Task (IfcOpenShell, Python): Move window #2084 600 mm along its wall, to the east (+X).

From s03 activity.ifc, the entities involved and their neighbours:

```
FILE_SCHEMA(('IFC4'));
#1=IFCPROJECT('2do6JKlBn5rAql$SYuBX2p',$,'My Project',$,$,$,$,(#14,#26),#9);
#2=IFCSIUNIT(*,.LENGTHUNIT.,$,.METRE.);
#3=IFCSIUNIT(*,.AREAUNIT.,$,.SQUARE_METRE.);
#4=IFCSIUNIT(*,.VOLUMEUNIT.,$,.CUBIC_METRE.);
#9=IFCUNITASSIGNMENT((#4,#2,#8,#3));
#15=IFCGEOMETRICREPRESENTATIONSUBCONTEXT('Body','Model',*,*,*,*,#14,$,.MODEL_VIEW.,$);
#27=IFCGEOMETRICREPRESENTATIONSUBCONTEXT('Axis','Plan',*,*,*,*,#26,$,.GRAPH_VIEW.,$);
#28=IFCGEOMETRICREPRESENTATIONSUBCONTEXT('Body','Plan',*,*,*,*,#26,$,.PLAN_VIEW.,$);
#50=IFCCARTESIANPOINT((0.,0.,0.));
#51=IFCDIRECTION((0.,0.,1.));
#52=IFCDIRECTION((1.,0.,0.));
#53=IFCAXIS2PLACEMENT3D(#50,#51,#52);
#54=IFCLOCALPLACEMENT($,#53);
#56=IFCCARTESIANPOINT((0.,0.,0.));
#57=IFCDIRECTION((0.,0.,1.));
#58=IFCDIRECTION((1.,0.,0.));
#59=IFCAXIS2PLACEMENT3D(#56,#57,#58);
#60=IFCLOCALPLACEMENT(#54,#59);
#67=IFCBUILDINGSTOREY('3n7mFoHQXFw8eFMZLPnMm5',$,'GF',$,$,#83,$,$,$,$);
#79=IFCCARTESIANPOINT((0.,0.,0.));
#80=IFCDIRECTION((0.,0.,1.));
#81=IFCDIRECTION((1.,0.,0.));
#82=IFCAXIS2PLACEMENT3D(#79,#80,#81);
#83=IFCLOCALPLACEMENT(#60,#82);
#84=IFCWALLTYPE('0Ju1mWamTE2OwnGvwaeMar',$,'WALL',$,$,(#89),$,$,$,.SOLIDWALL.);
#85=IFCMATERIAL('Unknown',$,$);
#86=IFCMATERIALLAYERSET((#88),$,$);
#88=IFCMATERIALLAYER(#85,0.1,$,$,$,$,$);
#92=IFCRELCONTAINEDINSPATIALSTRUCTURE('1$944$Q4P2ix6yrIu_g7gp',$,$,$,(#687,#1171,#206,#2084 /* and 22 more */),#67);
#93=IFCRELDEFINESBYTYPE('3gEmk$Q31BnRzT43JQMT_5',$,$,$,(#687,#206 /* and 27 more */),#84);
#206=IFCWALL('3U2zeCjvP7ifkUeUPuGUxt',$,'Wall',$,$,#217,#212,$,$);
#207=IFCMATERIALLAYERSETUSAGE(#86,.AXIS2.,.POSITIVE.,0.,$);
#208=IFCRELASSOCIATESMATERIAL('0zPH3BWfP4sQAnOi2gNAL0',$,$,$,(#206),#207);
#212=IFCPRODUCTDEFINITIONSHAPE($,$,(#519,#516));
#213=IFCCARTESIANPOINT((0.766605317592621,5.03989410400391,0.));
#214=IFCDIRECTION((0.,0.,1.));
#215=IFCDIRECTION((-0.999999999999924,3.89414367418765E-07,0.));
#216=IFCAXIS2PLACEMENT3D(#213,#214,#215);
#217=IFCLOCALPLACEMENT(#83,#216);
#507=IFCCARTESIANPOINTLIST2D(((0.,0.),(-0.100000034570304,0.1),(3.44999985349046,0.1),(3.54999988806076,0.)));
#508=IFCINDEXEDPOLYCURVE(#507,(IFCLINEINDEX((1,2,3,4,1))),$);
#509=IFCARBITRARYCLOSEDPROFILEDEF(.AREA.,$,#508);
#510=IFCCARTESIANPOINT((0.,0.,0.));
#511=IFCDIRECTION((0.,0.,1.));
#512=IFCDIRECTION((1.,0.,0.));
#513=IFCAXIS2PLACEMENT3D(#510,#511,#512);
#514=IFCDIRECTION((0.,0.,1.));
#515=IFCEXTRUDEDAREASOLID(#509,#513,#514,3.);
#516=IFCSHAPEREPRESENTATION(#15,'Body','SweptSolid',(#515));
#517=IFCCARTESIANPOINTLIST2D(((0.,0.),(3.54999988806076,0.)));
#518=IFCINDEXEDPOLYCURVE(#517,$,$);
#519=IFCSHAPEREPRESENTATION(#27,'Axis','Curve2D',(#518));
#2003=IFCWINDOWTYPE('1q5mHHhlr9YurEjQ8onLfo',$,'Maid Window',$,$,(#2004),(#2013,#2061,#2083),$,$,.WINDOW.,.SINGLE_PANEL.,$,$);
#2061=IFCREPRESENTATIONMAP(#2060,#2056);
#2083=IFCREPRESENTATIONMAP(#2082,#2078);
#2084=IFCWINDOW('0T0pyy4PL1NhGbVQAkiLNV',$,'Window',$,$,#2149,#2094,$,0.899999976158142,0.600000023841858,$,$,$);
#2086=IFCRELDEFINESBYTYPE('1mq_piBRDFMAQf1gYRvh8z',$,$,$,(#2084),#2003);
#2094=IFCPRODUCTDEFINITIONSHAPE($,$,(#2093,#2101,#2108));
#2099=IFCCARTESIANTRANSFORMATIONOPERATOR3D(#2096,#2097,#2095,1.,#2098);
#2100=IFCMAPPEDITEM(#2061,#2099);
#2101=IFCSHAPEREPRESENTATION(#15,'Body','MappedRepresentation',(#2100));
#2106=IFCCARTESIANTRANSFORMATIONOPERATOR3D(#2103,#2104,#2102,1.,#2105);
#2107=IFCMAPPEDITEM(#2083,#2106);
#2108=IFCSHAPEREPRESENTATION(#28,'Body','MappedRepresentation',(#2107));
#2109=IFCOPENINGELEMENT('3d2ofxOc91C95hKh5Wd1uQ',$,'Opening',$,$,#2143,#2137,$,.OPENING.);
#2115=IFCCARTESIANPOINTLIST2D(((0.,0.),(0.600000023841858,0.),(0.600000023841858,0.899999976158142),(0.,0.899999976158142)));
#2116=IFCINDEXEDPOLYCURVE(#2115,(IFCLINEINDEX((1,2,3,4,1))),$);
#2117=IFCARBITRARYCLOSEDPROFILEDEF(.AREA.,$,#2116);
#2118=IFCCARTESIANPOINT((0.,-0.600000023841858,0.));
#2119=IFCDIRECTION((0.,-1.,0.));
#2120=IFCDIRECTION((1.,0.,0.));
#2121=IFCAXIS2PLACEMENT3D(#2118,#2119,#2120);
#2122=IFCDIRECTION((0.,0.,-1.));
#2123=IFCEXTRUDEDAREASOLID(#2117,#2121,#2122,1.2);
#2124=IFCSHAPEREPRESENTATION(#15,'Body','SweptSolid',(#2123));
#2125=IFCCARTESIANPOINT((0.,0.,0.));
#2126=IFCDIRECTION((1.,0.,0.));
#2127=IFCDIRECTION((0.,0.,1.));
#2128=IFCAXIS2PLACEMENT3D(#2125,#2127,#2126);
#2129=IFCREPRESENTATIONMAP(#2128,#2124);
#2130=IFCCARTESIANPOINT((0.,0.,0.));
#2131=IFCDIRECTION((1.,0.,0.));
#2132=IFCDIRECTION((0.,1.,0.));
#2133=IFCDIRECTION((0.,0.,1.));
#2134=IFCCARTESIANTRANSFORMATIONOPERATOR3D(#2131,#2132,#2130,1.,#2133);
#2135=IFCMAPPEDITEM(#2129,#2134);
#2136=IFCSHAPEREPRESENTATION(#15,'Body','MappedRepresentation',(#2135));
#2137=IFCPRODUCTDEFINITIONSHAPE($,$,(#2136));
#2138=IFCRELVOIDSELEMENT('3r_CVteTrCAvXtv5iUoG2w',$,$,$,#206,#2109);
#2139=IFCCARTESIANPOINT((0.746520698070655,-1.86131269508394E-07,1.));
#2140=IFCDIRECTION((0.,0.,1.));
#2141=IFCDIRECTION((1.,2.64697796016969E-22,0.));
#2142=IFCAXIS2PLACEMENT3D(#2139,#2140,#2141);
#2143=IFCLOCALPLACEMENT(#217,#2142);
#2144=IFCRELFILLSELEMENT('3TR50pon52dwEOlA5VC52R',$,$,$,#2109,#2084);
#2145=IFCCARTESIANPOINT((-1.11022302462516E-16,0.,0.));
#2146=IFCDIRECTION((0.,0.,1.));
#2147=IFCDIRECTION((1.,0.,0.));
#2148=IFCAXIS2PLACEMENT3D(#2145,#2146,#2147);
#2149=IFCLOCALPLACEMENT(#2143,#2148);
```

```python
import ifcopenshell
import ifcopenshell.api.geometry
import ifcopenshell.util.placement
import ifcopenshell.util.unit

model = ifcopenshell.open("s03 activity.ifc")
unit_scale = ifcopenshell.util.unit.calculate_unit_scale(model)

window = model.by_guid("0T0pyy4PL1NhGbVQAkiLNV")
opening = window.FillsVoids[0].RelatingOpeningElement
wall = opening.VoidsElements[0].RelatingBuildingElement

wall_matrix = ifcopenshell.util.placement.get_local_placement(wall.ObjectPlacement)
shift = wall_matrix[:3, 0] * -0.6 / unit_scale
before = ifcopenshell.util.placement.get_local_placement(window.ObjectPlacement)[:3, 3].copy()

# The window is placed relative to its opening, so it follows when the opening moves.
matrix = ifcopenshell.util.placement.get_local_placement(opening.ObjectPlacement)
matrix[:3, 3] += shift
ifcopenshell.api.geometry.edit_object_placement(
    model, product=opening, matrix=matrix, is_si=False, should_transform_children=True
)

after = ifcopenshell.util.placement.get_local_placement(window.ObjectPlacement)[:3, 3]
print("window moved by", (after - before).round(3) + 0.0)

model.write("s03 activity-out.ifc")
```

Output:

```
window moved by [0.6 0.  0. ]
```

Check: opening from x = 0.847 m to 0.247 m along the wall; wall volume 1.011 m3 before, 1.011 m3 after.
